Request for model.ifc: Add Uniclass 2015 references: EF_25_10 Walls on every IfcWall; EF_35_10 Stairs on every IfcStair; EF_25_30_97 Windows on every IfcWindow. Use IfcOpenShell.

First a look at what the model holds.

```python
import ifcopenshell

model = ifcopenshell.open("model.ifc")
print(model.schema)
print("classifications:", [c.Name for c in model.by_type("IfcClassification")])
for ifc_class in ("IfcDoor", "IfcRoof", "IfcStair", "IfcWall", "IfcWindow"):
    print(ifc_class, len(model.by_type(ifc_class)))
```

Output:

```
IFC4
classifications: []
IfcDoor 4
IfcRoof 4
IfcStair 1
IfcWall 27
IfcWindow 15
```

```python
import ifcopenshell
import ifcopenshell.api.classification

model = ifcopenshell.open("model.ifc")

system = ifcopenshell.api.classification.add_classification(model, classification="Uniclass 2015")

codes = {
    "IfcWall": ("EF_25_10", "Walls"),
    "IfcStair": ("EF_35_10", "Stairs"),
    "IfcWindow": ("EF_25_30_97", "Windows"),
}
for ifc_class, (code, name) in codes.items():
    products = model.by_type(ifc_class)
    ifcopenshell.api.classification.add_reference(
        model, products=products, classification=system, identification=code, name=name
    )
    print(code, len(products))

model.write("model_edited.ifc")
```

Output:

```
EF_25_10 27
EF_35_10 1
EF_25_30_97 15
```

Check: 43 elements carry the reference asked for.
